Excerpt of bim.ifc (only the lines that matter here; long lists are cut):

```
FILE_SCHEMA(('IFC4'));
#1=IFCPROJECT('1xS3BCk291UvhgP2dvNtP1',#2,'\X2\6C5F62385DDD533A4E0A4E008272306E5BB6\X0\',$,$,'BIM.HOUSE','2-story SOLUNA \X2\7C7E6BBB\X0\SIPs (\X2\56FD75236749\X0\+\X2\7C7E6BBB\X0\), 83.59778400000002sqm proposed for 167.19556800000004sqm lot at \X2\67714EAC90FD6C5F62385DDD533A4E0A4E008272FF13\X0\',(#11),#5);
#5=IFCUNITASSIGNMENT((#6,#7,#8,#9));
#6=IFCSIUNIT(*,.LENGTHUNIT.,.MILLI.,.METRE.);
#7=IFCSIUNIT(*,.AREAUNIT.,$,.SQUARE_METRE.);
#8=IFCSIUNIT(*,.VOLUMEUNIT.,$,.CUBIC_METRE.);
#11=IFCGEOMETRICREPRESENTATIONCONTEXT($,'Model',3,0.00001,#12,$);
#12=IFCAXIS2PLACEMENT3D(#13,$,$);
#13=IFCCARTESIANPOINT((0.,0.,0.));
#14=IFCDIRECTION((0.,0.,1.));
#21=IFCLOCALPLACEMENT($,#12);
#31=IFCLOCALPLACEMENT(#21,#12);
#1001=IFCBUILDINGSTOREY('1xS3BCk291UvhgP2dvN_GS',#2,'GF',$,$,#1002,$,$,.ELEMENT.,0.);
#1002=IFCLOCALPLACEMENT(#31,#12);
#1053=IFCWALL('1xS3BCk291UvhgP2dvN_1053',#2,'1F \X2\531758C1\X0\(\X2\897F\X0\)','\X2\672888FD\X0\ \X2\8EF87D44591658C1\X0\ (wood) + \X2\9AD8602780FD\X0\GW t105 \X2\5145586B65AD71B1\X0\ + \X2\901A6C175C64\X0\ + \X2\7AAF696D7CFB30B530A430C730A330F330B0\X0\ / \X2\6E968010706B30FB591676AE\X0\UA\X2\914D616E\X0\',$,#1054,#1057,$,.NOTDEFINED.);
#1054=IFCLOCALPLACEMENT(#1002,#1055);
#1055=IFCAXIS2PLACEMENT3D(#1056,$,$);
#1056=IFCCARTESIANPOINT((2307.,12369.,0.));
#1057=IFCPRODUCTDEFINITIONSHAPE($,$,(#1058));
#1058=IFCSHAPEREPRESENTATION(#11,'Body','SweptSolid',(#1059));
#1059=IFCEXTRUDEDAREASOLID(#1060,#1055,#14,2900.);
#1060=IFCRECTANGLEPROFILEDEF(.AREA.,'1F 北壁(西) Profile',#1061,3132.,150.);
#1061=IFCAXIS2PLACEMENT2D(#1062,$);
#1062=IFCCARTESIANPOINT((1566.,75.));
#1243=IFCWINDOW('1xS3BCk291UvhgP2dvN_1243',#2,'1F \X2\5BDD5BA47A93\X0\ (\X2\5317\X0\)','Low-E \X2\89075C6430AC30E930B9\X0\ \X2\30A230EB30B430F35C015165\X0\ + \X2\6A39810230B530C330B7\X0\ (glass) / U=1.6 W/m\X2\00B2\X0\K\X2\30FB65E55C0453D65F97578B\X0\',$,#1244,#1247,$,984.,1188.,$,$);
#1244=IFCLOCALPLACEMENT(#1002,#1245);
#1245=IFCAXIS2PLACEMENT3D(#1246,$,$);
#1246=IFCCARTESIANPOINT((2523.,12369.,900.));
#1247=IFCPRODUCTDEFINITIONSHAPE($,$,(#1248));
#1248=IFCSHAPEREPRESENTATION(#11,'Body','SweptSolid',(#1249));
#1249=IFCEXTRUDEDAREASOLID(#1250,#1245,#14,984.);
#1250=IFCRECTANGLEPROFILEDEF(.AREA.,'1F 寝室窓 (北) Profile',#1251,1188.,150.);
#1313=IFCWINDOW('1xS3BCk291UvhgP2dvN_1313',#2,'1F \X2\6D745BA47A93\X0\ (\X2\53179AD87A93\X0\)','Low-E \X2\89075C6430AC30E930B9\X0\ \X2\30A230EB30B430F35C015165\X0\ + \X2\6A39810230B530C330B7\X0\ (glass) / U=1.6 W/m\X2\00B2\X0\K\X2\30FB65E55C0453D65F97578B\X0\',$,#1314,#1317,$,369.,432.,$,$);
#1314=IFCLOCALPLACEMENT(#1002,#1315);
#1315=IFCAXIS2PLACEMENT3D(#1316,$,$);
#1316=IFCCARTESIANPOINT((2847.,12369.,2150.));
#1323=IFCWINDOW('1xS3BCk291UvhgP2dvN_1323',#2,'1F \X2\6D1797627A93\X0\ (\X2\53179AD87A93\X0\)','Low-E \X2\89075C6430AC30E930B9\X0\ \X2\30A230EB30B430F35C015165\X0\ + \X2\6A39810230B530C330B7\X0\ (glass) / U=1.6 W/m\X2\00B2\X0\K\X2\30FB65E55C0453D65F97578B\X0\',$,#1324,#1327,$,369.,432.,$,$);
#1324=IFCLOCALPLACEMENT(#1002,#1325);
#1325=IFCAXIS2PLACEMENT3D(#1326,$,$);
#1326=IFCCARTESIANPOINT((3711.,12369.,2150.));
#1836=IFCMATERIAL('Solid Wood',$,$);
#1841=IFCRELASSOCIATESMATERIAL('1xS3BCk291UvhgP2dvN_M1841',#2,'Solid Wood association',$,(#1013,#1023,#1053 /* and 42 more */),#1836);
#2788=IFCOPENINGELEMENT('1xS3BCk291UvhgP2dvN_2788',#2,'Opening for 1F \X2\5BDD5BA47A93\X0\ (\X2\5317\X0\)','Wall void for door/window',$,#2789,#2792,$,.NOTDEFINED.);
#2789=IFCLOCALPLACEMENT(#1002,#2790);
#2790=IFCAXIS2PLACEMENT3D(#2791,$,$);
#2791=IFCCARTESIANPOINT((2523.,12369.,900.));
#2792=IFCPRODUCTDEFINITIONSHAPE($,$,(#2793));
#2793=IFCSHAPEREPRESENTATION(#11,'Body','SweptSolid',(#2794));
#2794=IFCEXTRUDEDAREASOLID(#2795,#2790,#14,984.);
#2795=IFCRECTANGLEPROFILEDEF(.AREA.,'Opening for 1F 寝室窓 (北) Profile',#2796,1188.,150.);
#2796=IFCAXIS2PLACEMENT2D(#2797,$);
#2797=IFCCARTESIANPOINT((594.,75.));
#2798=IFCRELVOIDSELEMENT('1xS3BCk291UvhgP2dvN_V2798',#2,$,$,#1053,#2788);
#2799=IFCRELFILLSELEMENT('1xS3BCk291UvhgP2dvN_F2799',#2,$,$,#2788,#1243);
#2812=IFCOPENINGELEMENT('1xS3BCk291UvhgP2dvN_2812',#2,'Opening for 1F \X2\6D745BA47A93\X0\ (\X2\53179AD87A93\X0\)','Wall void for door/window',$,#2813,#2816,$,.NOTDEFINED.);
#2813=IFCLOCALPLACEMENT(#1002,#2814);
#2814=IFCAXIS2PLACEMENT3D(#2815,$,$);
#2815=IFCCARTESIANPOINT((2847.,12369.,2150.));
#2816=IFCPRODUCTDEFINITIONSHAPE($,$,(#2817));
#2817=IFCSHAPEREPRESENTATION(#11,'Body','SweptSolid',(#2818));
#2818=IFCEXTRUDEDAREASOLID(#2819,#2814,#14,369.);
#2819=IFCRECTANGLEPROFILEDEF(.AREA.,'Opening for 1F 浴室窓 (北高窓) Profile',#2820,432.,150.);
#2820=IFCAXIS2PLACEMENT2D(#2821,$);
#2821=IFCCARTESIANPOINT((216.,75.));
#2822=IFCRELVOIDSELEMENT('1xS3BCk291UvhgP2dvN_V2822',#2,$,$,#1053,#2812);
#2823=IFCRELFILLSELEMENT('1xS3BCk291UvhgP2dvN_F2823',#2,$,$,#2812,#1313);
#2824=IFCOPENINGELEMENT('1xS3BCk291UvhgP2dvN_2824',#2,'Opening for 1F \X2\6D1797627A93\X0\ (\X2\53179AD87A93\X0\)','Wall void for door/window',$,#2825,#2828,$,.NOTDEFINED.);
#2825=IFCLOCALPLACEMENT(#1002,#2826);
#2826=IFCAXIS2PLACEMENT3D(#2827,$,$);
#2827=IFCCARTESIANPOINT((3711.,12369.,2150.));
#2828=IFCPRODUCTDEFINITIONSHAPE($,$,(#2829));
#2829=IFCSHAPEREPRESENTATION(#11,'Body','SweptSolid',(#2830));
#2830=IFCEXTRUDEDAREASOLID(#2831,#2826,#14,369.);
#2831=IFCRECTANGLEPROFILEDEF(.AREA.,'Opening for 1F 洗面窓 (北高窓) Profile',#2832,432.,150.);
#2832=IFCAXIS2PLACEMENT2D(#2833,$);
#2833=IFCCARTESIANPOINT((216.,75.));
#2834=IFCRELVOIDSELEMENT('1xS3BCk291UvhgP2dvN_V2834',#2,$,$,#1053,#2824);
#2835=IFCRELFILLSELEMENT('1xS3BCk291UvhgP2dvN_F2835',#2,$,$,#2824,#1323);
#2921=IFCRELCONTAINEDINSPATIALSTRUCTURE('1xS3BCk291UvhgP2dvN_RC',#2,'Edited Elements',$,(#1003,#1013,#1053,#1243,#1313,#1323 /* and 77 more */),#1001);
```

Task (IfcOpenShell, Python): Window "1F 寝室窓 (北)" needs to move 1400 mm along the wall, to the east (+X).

```python
import ifcopenshell
import ifcopenshell.api.geometry
import ifcopenshell.util.placement
import ifcopenshell.util.unit

model = ifcopenshell.open("bim.ifc")
unit_scale = ifcopenshell.util.unit.calculate_unit_scale(model)

window = model.by_id(1243)
opening = window.FillsVoids[0].RelatingOpeningElement
wall = opening.VoidsElements[0].RelatingBuildingElement

wall_matrix = ifcopenshell.util.placement.get_local_placement(wall.ObjectPlacement)
shift = wall_matrix[:3, 0] * 1.4 / unit_scale
before = ifcopenshell.util.placement.get_local_placement(window.ObjectPlacement)[:3, 3].copy()

# The window is not placed relative to its opening, so move both.
for product in (opening, window):
    matrix = ifcopenshell.util.placement.get_local_placement(product.ObjectPlacement)
    matrix[:3, 3] += shift
    ifcopenshell.api.geometry.edit_object_placement(model, product=product, matrix=matrix, is_si=False)

after = ifcopenshell.util.placement.get_local_placement(window.ObjectPlacement)[:3, 3]
print("window moved by", (after - before).round(3) + 0.0)

model.write("bim_v2.ifc")
```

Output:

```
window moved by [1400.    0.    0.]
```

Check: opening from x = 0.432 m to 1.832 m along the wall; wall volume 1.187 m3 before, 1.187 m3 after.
